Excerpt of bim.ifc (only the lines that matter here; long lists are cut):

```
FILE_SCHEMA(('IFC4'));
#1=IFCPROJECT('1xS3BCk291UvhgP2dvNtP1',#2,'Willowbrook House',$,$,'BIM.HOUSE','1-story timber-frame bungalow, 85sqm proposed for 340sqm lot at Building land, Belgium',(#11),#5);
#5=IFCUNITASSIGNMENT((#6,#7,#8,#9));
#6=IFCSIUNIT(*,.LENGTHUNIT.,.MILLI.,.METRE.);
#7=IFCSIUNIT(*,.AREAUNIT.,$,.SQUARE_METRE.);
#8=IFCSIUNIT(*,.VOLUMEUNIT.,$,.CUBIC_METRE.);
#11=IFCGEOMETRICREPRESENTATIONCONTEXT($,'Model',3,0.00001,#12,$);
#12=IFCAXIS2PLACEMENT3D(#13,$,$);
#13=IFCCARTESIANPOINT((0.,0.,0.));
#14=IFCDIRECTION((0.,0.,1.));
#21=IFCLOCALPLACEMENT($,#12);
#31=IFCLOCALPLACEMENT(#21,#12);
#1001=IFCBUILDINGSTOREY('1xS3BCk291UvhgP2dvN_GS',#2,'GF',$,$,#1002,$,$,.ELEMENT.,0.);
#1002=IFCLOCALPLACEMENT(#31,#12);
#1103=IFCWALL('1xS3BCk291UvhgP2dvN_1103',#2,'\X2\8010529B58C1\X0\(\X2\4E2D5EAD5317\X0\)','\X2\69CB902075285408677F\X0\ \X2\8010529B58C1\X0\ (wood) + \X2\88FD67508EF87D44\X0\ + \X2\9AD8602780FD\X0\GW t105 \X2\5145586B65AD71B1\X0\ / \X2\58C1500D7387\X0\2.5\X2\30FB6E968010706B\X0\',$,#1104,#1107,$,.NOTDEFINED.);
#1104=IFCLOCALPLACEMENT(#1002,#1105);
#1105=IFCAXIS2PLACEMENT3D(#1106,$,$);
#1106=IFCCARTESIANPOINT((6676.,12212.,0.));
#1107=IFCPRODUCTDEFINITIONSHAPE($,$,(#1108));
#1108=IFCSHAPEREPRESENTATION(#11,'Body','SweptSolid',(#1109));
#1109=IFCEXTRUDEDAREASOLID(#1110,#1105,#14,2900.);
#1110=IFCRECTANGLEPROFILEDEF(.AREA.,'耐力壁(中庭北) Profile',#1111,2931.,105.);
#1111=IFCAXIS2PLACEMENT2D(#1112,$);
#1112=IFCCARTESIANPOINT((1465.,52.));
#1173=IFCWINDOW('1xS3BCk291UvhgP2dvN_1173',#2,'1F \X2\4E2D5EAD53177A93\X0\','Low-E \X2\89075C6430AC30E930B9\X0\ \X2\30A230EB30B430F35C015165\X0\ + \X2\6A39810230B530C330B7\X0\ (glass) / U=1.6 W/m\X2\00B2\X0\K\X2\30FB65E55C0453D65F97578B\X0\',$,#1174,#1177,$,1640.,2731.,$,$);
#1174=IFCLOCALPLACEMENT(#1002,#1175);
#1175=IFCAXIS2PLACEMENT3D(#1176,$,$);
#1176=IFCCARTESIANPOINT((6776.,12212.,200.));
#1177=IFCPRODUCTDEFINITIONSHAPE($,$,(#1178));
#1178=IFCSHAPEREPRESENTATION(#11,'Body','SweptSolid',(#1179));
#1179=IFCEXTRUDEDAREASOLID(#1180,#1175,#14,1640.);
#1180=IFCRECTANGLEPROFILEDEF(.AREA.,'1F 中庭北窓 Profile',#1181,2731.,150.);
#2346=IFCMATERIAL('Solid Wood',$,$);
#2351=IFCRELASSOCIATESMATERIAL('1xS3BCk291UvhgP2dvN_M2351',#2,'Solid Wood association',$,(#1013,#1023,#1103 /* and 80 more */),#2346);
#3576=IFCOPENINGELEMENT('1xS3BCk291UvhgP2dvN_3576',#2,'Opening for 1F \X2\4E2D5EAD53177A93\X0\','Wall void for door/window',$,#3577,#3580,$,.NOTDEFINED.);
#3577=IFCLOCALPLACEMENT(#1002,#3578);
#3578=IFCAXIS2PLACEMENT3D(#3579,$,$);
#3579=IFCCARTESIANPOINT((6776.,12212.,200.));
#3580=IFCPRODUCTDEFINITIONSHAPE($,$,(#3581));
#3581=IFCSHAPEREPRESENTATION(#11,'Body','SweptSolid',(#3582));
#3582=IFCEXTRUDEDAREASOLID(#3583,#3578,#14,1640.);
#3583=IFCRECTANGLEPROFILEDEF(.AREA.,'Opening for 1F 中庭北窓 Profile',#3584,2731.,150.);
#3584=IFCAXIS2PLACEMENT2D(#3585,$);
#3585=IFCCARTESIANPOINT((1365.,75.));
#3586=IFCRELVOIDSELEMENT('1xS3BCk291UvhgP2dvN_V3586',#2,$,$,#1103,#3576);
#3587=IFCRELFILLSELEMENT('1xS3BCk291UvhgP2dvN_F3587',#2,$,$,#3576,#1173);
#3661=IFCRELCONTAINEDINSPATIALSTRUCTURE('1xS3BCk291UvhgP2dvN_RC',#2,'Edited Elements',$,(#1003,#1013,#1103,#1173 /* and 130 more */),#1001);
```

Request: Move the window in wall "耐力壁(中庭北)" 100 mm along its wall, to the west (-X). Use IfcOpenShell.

```python
import ifcopenshell
import ifcopenshell.api.geometry
import ifcopenshell.util.placement
import ifcopenshell.util.unit

model = ifcopenshell.open("bim.ifc")
unit_scale = ifcopenshell.util.unit.calculate_unit_scale(model)

window = model.by_id(1173)
opening = window.FillsVoids[0].RelatingOpeningElement
wall = opening.VoidsElements[0].RelatingBuildingElement

wall_matrix = ifcopenshell.util.placement.get_local_placement(wall.ObjectPlacement)
shift = wall_matrix[:3, 0] * -0.1 / unit_scale
before = ifcopenshell.util.placement.get_local_placement(window.ObjectPlacement)[:3, 3].copy()

# The window is not placed relative to its opening, so move both.
for product in (opening, window):
    matrix = ifcopenshell.util.placement.get_local_placement(product.ObjectPlacement)
    matrix[:3, 3] += shift
    ifcopenshell.api.geometry.edit_object_placement(model, product=product, matrix=matrix, is_si=False)

after = ifcopenshell.util.placement.get_local_placement(window.ObjectPlacement)[:3, 3]
print("window moved by", (after - before).round(3) + 0.0)

model.write("bim_edited.ifc")
```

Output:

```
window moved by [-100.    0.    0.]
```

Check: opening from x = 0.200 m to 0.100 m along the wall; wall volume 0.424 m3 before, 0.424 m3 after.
